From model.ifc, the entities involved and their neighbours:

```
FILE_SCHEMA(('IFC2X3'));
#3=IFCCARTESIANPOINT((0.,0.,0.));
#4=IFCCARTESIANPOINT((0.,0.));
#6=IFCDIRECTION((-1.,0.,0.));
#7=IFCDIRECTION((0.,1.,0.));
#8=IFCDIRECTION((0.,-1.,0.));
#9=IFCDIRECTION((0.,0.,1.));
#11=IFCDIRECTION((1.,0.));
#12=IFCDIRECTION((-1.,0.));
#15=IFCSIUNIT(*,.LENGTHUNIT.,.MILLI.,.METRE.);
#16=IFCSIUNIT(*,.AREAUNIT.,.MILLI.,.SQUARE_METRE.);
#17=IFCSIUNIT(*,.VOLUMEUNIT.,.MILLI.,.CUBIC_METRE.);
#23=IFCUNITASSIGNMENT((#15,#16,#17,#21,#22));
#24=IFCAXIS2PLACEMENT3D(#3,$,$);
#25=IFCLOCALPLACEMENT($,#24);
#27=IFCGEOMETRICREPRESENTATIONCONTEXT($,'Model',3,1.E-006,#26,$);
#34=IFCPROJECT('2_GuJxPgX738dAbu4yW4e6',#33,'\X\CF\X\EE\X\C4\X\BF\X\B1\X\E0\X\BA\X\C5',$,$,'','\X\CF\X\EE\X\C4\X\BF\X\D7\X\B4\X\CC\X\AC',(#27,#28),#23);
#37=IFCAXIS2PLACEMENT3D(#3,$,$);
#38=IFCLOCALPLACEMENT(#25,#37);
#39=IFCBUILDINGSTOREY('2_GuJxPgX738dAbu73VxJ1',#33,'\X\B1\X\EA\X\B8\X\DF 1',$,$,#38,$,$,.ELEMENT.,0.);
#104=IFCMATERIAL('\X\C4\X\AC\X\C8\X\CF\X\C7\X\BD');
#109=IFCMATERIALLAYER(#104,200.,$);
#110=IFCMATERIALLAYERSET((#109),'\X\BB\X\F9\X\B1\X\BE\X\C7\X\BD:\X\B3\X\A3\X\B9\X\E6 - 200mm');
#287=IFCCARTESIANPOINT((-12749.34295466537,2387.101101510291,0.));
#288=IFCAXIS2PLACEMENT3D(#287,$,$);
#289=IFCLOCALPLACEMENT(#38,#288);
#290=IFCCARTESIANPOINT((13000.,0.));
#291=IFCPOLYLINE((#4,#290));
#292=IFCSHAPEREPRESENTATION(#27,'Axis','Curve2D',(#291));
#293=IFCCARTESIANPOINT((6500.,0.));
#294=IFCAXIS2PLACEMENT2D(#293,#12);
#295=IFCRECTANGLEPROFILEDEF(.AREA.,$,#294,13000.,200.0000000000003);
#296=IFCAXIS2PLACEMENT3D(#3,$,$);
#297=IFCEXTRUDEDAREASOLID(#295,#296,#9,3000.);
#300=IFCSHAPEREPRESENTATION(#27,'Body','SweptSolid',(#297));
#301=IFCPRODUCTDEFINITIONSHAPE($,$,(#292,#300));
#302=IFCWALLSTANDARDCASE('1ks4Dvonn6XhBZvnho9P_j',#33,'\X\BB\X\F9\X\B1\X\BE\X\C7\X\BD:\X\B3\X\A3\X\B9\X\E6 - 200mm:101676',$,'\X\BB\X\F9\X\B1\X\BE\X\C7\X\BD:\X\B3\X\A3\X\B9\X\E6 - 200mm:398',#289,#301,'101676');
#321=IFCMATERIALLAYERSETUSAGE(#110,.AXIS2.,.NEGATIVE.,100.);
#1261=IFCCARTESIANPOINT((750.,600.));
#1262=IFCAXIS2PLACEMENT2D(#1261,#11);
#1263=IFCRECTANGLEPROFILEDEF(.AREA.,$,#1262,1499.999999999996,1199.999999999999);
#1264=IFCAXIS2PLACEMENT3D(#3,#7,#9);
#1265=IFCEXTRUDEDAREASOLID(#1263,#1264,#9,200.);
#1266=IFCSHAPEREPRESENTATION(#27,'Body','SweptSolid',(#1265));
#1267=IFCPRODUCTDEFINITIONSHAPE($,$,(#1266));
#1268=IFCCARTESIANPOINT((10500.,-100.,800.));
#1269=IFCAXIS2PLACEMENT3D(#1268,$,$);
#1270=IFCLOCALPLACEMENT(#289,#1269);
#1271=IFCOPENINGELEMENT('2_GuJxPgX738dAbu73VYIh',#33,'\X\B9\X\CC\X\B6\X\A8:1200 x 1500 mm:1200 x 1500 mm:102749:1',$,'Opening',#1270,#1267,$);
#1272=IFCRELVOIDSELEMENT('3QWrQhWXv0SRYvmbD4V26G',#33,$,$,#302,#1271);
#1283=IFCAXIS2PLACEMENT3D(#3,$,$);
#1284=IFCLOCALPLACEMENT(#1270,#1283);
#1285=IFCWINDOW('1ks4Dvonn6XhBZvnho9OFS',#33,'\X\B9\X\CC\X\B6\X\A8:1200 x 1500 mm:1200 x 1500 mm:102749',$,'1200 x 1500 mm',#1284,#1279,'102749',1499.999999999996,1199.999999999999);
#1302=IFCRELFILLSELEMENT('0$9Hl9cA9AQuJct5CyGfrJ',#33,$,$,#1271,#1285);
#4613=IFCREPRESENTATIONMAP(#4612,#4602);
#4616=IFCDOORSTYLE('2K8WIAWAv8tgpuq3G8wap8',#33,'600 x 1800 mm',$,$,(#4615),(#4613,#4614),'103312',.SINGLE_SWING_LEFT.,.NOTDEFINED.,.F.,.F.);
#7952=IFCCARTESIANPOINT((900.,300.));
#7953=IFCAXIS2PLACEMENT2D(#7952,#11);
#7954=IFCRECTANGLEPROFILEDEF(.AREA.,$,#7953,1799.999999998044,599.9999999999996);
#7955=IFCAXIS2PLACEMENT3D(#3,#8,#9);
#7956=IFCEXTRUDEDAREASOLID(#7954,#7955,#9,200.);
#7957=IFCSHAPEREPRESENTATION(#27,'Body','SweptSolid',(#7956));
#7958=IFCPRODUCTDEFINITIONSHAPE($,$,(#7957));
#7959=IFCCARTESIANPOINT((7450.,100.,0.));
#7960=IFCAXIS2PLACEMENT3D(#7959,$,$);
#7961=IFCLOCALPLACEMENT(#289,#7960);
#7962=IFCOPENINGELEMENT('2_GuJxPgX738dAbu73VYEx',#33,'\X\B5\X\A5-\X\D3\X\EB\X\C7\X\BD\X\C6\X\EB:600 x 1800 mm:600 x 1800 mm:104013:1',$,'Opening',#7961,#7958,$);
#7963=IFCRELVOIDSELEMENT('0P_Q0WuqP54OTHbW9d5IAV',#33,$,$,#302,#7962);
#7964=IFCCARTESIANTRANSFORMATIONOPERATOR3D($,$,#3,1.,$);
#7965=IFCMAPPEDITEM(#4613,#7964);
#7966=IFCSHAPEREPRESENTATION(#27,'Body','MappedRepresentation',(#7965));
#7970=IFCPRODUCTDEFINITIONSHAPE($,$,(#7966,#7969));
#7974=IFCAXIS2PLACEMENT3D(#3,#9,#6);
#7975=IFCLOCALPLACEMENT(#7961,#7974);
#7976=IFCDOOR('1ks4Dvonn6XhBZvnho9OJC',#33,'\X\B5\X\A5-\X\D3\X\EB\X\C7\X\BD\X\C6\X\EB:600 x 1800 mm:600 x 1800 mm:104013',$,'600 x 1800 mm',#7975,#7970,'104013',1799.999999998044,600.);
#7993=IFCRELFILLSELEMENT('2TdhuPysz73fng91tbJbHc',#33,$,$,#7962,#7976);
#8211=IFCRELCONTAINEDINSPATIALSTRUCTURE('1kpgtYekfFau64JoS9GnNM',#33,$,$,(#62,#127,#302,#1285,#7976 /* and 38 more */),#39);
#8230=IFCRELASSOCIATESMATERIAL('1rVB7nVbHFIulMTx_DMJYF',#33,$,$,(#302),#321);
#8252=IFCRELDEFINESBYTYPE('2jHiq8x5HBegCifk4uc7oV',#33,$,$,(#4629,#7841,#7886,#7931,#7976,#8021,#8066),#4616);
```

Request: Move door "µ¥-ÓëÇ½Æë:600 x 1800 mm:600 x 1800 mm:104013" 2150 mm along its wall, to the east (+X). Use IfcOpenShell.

```python
import ifcopenshell
import ifcopenshell.api.geometry
import ifcopenshell.util.placement
import ifcopenshell.util.unit

model = ifcopenshell.open("model.ifc")
unit_scale = ifcopenshell.util.unit.calculate_unit_scale(model)

door = model.by_guid("1ks4Dvonn6XhBZvnho9OJC")
opening = door.FillsVoids[0].RelatingOpeningElement
wall = opening.VoidsElements[0].RelatingBuildingElement

wall_matrix = ifcopenshell.util.placement.get_local_placement(wall.ObjectPlacement)
shift = wall_matrix[:3, 0] * 2.15 / unit_scale
before = ifcopenshell.util.placement.get_local_placement(door.ObjectPlacement)[:3, 3].copy()

# The door is placed relative to its opening, so it follows when the opening moves.
matrix = ifcopenshell.util.placement.get_local_placement(opening.ObjectPlacement)
matrix[:3, 3] += shift
ifcopenshell.api.geometry.edit_object_placement(
    model, product=opening, matrix=matrix, is_si=False, should_transform_children=True
)

after = ifcopenshell.util.placement.get_local_placement(door.ObjectPlacement)[:3, 3]
print("door moved by", (after - before).round(3) + 0.0)

model.write("model_v2.ifc")
```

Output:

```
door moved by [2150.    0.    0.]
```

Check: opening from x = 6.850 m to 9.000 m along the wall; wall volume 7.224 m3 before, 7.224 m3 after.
